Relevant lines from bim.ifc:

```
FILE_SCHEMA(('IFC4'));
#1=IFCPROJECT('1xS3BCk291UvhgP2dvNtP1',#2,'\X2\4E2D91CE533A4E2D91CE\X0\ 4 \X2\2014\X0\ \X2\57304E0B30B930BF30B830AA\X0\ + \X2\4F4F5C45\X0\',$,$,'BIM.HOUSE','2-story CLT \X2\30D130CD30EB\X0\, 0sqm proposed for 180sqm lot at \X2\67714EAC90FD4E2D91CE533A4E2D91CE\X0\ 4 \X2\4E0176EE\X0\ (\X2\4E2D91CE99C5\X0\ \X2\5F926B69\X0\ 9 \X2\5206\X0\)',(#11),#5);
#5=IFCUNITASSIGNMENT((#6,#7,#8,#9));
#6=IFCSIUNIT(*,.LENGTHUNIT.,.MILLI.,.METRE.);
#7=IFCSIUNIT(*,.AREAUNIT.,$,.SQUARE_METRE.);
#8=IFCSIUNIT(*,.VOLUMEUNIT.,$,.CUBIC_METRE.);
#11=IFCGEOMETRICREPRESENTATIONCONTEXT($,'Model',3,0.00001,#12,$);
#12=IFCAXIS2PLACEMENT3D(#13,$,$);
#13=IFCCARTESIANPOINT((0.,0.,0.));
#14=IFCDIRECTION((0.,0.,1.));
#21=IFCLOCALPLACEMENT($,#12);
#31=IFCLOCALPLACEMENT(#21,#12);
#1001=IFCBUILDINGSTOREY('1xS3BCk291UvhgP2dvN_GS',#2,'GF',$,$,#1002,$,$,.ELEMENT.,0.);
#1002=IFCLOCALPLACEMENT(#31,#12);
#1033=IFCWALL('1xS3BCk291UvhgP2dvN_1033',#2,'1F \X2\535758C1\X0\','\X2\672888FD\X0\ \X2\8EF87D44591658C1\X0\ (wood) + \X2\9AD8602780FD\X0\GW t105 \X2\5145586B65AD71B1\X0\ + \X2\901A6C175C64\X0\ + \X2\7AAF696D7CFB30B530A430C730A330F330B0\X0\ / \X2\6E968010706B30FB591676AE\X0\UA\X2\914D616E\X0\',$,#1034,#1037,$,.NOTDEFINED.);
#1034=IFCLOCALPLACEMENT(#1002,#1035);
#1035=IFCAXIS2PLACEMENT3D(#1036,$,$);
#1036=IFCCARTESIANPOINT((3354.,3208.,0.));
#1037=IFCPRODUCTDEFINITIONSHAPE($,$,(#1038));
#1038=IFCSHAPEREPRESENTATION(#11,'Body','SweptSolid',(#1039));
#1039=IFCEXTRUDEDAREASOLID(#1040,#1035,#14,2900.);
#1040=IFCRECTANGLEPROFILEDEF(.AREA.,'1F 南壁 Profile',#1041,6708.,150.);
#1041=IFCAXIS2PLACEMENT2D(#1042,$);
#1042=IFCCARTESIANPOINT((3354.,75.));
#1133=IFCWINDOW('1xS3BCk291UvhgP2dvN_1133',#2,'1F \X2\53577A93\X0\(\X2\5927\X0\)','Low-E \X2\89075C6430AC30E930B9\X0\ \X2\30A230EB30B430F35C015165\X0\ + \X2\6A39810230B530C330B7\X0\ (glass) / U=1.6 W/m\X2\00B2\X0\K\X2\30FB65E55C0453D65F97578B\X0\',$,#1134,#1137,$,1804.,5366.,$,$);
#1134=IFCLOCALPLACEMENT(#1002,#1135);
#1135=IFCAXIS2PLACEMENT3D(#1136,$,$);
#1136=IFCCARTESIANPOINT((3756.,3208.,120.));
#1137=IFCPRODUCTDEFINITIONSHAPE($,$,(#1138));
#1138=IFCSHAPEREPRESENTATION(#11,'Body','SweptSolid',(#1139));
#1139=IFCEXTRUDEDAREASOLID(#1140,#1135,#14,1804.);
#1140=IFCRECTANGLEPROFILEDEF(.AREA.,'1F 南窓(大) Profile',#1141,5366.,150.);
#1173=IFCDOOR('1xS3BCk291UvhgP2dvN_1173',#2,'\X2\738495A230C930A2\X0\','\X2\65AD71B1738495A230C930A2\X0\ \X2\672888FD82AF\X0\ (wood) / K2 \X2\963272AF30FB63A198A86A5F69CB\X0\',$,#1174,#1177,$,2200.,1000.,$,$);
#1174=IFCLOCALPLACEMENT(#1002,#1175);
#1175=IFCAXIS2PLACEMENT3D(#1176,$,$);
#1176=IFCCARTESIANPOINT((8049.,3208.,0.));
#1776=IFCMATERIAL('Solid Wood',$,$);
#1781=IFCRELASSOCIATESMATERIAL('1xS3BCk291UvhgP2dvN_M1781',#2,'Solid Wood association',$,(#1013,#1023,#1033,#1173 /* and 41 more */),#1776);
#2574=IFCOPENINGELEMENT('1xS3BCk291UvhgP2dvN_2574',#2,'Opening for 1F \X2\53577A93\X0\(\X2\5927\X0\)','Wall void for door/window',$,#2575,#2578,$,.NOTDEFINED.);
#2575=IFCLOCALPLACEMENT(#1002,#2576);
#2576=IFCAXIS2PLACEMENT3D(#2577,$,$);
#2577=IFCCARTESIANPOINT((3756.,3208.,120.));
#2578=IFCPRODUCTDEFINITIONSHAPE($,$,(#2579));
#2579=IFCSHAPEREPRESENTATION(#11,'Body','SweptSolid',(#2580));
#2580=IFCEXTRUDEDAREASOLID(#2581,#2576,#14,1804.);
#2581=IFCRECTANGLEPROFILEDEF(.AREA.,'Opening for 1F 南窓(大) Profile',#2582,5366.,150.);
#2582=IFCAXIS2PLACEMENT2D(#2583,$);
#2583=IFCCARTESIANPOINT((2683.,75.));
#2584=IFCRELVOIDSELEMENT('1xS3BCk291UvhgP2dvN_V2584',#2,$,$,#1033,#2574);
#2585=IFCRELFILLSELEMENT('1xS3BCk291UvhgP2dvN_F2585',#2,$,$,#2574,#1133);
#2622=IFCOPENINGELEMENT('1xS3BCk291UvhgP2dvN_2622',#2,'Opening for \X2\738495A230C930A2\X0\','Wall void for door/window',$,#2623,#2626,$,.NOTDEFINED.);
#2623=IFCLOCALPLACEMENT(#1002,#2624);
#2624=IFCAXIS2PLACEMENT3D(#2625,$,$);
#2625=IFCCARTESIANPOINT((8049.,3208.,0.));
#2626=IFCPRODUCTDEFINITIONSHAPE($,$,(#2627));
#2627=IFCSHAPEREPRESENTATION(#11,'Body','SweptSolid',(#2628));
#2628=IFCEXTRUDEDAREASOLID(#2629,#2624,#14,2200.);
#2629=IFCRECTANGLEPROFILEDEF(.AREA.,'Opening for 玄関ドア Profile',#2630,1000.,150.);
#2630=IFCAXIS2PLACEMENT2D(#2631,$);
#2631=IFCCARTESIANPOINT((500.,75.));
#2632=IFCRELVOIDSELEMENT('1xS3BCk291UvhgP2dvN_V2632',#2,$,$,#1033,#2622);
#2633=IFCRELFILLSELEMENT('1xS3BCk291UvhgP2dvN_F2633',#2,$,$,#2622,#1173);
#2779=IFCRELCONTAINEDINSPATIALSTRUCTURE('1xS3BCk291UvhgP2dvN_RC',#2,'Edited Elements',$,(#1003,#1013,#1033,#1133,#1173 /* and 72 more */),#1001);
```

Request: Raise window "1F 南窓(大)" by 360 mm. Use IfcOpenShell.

```python
import numpy as np
import ifcopenshell
import ifcopenshell.api.geometry
import ifcopenshell.util.placement
import ifcopenshell.util.unit

model = ifcopenshell.open("bim.ifc")
unit_scale = ifcopenshell.util.unit.calculate_unit_scale(model)

window = model.by_guid("1xS3BCk291UvhgP2dvN_1133")
opening = window.FillsVoids[0].RelatingOpeningElement
dz = 360.0

shift = np.array([0.0, 0.0, dz])
# The window is not placed relative to its opening, so move both.
for product in (opening, window):
    matrix = ifcopenshell.util.placement.get_local_placement(product.ObjectPlacement)
    matrix[:3, 3] += shift
    ifcopenshell.api.geometry.edit_object_placement(model, product=product, matrix=matrix, is_si=False)

print(f"moved by {dz * unit_scale:+.3f} m")

model.write("bim_updated.ifc")
```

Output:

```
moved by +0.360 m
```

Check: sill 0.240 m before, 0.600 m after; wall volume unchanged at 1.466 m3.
